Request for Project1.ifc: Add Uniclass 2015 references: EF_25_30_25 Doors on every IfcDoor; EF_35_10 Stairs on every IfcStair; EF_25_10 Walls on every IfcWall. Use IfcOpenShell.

First a look at what the model holds.

```python
import ifcopenshell

model = ifcopenshell.open("Project1.ifc")
print(model.schema)
print("classifications:", [c.Name for c in model.by_type("IfcClassification")])
for ifc_class in ("IfcDoor", "IfcRoof", "IfcStair", "IfcWall", "IfcWindow"):
    print(ifc_class, len(model.by_type(ifc_class)))
```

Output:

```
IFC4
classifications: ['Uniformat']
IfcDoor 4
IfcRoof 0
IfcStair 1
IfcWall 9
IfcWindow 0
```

```python
import ifcopenshell
import ifcopenshell.api.classification

model = ifcopenshell.open("Project1.ifc")

system = ifcopenshell.api.classification.add_classification(model, classification="Uniclass 2015")

codes = {
    "IfcDoor": ("EF_25_30_25", "Doors"),
    "IfcStair": ("EF_35_10", "Stairs"),
    "IfcWall": ("EF_25_10", "Walls"),
}
for ifc_class, (code, name) in codes.items():
    products = model.by_type(ifc_class)
    ifcopenshell.api.classification.add_reference(
        model, products=products, classification=system, identification=code, name=name
    )
    print(code, len(products))

model.write("Project1-out.ifc")
```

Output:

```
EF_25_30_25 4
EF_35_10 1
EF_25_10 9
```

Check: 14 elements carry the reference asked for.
